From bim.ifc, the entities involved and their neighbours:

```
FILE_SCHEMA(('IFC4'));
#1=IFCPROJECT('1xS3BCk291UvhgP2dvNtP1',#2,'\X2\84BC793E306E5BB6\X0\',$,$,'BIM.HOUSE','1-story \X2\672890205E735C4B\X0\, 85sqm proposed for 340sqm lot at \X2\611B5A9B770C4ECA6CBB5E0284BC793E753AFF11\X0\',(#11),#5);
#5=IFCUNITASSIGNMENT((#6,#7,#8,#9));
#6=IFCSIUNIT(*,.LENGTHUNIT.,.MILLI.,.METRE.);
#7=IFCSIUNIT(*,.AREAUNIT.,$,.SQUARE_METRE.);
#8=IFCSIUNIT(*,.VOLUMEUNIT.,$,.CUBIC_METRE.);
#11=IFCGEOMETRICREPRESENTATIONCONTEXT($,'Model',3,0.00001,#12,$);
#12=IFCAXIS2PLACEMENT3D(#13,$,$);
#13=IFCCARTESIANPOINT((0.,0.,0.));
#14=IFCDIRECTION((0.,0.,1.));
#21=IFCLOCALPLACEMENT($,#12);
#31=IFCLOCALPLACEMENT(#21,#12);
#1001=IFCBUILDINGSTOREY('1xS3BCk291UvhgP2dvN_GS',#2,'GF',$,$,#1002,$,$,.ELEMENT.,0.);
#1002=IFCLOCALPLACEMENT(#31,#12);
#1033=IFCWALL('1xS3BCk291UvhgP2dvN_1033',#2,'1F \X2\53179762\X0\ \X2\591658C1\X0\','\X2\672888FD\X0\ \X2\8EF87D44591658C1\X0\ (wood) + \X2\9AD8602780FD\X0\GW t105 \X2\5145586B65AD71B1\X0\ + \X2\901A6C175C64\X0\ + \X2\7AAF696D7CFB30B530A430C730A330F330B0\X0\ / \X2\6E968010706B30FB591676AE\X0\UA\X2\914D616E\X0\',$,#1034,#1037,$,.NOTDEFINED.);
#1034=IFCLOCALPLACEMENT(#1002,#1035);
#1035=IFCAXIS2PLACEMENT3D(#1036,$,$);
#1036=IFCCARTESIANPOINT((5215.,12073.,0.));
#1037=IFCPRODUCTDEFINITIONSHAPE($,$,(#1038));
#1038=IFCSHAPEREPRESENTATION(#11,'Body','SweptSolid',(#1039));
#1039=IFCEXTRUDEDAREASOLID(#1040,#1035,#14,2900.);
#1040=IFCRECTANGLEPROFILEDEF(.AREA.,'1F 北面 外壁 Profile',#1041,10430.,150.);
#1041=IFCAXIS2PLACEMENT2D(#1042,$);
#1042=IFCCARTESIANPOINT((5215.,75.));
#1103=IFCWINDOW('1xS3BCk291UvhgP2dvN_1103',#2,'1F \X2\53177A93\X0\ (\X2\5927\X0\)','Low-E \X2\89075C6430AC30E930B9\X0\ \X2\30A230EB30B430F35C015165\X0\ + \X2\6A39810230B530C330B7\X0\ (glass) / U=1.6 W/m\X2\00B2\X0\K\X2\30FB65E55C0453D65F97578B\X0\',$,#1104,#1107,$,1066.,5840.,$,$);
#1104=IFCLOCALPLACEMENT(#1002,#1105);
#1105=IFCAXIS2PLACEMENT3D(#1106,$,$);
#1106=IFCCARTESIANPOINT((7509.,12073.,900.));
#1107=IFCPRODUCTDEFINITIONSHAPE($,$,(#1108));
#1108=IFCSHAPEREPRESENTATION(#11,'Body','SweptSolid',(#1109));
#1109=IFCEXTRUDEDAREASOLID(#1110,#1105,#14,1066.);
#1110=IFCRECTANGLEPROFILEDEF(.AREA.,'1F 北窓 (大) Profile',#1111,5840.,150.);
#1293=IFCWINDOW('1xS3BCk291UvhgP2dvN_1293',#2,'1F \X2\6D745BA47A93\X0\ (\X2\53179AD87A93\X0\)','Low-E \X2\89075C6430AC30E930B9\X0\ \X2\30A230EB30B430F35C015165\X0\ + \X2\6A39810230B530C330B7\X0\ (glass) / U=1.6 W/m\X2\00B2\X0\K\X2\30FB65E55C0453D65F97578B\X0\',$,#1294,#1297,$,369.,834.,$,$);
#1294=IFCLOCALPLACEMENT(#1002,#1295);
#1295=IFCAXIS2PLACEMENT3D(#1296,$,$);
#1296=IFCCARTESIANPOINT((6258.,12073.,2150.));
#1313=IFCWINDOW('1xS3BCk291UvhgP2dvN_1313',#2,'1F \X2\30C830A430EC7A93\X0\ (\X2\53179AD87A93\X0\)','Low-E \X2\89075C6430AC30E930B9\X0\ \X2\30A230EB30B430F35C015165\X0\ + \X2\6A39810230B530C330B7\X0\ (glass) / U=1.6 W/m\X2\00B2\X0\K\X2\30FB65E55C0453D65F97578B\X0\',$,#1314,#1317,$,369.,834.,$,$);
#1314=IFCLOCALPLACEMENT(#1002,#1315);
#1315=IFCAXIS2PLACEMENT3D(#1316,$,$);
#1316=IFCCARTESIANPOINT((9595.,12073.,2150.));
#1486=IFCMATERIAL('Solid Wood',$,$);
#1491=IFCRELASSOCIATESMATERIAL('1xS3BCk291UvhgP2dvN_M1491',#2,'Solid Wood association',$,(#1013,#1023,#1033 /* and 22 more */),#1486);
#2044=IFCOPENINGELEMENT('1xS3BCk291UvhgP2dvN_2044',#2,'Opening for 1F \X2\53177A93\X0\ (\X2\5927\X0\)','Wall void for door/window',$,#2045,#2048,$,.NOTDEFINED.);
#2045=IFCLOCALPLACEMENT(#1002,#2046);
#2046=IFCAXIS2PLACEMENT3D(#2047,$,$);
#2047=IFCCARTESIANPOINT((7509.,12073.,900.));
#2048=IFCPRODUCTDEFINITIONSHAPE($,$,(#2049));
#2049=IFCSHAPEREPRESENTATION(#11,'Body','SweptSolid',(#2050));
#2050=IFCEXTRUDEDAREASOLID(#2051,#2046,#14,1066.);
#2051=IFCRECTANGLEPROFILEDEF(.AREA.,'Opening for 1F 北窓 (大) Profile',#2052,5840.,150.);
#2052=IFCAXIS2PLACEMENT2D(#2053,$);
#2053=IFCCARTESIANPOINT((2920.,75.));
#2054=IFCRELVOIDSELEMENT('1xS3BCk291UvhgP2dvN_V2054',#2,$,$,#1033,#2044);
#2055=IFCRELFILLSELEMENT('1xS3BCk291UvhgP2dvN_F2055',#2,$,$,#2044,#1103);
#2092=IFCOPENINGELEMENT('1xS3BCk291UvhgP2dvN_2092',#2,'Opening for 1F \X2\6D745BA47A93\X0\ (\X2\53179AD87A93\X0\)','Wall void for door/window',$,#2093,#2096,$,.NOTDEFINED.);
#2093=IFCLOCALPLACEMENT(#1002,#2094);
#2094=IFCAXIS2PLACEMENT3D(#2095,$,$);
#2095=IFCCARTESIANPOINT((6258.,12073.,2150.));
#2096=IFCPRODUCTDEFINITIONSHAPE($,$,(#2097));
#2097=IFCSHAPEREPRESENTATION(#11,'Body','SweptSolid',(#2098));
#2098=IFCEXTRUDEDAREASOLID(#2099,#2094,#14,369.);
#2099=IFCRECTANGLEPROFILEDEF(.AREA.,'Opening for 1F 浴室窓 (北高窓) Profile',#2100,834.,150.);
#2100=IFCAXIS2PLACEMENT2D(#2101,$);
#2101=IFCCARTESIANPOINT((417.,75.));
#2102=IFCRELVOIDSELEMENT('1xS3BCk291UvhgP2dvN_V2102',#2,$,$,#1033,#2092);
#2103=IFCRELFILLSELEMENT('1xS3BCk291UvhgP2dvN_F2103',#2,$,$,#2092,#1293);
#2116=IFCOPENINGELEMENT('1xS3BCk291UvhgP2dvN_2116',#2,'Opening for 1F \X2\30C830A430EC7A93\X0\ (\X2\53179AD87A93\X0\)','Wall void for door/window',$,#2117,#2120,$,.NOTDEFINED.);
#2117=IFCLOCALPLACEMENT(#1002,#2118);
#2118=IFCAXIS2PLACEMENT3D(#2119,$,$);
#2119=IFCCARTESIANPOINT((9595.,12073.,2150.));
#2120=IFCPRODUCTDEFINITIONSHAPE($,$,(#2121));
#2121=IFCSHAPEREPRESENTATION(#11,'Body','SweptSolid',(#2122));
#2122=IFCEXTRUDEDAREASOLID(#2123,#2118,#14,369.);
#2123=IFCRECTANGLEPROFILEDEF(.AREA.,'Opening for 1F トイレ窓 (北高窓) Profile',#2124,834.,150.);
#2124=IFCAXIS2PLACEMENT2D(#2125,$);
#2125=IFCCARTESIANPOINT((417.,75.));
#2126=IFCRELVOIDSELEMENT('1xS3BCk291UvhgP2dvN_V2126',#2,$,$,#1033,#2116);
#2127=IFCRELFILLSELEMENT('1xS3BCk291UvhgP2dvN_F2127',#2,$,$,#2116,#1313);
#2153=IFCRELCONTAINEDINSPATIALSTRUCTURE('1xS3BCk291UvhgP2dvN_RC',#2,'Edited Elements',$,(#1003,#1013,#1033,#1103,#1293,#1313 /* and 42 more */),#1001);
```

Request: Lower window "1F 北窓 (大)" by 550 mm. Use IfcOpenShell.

```python
import numpy as np
import ifcopenshell
import ifcopenshell.api.geometry
import ifcopenshell.util.placement
import ifcopenshell.util.unit

model = ifcopenshell.open("bim.ifc")
unit_scale = ifcopenshell.util.unit.calculate_unit_scale(model)

window = model.by_guid("1xS3BCk291UvhgP2dvN_1103")
opening = window.FillsVoids[0].RelatingOpeningElement
dz = -0.55 / unit_scale

shift = np.array([0.0, 0.0, dz])
# The window is not placed relative to its opening, so move both.
for product in (opening, window):
    matrix = ifcopenshell.util.placement.get_local_placement(product.ObjectPlacement)
    matrix[:3, 3] += shift
    ifcopenshell.api.geometry.edit_object_placement(model, product=product, matrix=matrix, is_si=False)

print(f"moved by {dz * unit_scale:+.3f} m")

model.write("bim_rev.ifc")
```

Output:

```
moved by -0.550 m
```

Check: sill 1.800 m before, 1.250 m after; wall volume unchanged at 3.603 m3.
